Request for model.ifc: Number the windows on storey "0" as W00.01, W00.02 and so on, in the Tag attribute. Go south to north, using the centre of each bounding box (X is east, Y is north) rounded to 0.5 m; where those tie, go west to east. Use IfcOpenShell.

First a look at what the model holds.

```python
import ifcopenshell
import ifcopenshell.util.element
import ifcopenshell.util.placement

model = ifcopenshell.open("model.ifc")
print(model.schema)
storey = next(s for s in model.by_type("IfcBuildingStorey") if s.Name == "0")
windows = [e for e in ifcopenshell.util.element.get_decomposition(storey) if e.is_a("IfcWindow")]
for e in sorted(windows, key=lambda e: e.id()):
    origin = ifcopenshell.util.placement.get_local_placement(e.ObjectPlacement)[:3, 3]
    print(e.id(), e.Tag, e.Name, origin.round(2) + 0.0, sep=" | ")
```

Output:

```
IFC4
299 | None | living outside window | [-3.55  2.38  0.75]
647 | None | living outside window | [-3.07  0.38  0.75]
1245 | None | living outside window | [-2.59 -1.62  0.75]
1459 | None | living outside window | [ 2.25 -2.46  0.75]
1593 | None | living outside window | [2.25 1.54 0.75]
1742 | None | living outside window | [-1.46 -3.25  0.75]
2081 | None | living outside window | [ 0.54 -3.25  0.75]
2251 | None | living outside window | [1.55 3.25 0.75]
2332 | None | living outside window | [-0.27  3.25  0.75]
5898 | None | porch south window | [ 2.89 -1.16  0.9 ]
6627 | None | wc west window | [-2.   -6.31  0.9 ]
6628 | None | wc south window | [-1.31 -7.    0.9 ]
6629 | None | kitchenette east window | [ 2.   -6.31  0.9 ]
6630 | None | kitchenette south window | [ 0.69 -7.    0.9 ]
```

```python
import ifcopenshell
import ifcopenshell.geom
import ifcopenshell.util.element
import ifcopenshell.util.shape

model = ifcopenshell.open("model.ifc")
settings = ifcopenshell.geom.settings()
settings.set("use-world-coords", True)


def centre(element):
    shape = ifcopenshell.geom.create_shape(settings, element)
    return ifcopenshell.util.shape.get_bbox_centroid(shape.geometry)


storey = next(s for s in model.by_type("IfcBuildingStorey") if s.Name == "0")
windows = [e for e in ifcopenshell.util.element.get_decomposition(storey) if e.is_a("IfcWindow")]

# Insertion points can sit at a corner or the storey origin, so sort by the geometry (in metres).
centres = {e: centre(e) for e in windows}
windows.sort(key=lambda e: (round(centres[e][1] / 0.5), centres[e][0]))

for i, e in enumerate(windows, start=1):
    number = f"W00.{i:02d}"
    e.Tag = number
    print(e.id(), number)

model.write("model-out.ifc")
```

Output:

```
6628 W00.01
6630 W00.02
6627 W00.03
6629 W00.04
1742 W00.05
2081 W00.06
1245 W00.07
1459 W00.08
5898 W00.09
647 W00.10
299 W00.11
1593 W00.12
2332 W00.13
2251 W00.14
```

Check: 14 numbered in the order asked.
